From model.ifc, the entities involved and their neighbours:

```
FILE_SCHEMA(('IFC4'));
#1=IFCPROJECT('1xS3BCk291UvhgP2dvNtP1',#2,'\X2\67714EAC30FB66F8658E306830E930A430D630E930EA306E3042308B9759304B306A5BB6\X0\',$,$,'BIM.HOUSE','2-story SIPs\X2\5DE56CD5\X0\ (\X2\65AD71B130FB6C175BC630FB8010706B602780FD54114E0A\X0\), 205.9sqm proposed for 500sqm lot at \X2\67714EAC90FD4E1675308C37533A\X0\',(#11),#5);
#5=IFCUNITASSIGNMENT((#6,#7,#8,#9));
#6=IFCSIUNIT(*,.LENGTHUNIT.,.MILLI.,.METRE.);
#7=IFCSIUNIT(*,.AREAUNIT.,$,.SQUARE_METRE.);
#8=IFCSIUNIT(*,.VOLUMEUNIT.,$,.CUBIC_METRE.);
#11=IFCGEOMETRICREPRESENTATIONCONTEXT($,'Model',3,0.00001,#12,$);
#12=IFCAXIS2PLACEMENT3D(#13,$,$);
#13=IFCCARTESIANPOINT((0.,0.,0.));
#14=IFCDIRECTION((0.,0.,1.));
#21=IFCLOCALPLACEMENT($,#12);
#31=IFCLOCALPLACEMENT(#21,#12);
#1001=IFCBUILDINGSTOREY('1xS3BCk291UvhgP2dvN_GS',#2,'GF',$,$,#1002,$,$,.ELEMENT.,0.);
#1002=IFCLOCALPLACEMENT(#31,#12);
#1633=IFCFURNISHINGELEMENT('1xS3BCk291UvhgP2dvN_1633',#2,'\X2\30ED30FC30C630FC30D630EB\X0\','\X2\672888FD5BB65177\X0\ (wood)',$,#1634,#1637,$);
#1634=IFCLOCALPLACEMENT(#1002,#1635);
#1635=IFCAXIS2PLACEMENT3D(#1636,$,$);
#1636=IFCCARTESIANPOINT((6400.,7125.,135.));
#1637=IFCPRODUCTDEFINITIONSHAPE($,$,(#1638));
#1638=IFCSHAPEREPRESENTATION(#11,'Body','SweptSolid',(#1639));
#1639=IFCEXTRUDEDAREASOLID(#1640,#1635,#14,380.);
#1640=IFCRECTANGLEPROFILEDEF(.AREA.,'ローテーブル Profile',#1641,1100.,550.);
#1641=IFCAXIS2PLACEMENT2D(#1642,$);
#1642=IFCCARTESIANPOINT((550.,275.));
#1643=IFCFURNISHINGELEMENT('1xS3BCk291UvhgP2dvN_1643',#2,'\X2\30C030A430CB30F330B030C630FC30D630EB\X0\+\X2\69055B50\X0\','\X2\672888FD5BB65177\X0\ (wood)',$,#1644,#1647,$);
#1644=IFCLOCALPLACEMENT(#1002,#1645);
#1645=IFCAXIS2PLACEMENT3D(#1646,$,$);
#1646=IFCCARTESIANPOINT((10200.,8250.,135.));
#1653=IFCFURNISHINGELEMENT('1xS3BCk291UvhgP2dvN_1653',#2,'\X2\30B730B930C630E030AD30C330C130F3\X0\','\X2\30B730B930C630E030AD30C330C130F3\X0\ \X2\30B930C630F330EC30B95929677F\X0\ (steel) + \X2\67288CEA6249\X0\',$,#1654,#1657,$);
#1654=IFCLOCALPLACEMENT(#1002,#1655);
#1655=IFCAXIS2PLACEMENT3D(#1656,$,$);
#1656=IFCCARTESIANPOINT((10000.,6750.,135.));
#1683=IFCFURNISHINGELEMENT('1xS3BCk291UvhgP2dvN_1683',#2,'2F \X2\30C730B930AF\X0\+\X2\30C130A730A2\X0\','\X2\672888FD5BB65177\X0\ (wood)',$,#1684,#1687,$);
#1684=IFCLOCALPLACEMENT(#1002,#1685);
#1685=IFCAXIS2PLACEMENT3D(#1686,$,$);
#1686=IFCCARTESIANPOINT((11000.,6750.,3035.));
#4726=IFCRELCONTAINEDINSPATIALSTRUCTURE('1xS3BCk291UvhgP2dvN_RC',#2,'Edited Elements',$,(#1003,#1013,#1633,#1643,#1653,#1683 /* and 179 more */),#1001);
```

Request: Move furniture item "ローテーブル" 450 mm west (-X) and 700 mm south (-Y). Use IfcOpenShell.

```python
import ifcopenshell
import ifcopenshell.api.geometry
import ifcopenshell.util.placement
import ifcopenshell.util.unit

model = ifcopenshell.open("model.ifc")
unit_scale = ifcopenshell.util.unit.calculate_unit_scale(model)

item = model.by_guid("1xS3BCk291UvhgP2dvN_1633")
matrix = ifcopenshell.util.placement.get_local_placement(item.ObjectPlacement)
matrix[0, 3] -= 0.45 / unit_scale
matrix[1, 3] -= 0.7 / unit_scale
ifcopenshell.api.geometry.edit_object_placement(model, product=item, matrix=matrix, is_si=False)

print(ifcopenshell.util.placement.get_local_placement(item.ObjectPlacement).round(3) + 0.0)

model.write("model_edited.ifc")
```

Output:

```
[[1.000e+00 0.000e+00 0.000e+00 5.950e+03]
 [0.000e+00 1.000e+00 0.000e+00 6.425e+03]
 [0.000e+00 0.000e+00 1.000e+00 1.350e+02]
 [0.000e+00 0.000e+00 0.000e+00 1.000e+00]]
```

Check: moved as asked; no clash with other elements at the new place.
